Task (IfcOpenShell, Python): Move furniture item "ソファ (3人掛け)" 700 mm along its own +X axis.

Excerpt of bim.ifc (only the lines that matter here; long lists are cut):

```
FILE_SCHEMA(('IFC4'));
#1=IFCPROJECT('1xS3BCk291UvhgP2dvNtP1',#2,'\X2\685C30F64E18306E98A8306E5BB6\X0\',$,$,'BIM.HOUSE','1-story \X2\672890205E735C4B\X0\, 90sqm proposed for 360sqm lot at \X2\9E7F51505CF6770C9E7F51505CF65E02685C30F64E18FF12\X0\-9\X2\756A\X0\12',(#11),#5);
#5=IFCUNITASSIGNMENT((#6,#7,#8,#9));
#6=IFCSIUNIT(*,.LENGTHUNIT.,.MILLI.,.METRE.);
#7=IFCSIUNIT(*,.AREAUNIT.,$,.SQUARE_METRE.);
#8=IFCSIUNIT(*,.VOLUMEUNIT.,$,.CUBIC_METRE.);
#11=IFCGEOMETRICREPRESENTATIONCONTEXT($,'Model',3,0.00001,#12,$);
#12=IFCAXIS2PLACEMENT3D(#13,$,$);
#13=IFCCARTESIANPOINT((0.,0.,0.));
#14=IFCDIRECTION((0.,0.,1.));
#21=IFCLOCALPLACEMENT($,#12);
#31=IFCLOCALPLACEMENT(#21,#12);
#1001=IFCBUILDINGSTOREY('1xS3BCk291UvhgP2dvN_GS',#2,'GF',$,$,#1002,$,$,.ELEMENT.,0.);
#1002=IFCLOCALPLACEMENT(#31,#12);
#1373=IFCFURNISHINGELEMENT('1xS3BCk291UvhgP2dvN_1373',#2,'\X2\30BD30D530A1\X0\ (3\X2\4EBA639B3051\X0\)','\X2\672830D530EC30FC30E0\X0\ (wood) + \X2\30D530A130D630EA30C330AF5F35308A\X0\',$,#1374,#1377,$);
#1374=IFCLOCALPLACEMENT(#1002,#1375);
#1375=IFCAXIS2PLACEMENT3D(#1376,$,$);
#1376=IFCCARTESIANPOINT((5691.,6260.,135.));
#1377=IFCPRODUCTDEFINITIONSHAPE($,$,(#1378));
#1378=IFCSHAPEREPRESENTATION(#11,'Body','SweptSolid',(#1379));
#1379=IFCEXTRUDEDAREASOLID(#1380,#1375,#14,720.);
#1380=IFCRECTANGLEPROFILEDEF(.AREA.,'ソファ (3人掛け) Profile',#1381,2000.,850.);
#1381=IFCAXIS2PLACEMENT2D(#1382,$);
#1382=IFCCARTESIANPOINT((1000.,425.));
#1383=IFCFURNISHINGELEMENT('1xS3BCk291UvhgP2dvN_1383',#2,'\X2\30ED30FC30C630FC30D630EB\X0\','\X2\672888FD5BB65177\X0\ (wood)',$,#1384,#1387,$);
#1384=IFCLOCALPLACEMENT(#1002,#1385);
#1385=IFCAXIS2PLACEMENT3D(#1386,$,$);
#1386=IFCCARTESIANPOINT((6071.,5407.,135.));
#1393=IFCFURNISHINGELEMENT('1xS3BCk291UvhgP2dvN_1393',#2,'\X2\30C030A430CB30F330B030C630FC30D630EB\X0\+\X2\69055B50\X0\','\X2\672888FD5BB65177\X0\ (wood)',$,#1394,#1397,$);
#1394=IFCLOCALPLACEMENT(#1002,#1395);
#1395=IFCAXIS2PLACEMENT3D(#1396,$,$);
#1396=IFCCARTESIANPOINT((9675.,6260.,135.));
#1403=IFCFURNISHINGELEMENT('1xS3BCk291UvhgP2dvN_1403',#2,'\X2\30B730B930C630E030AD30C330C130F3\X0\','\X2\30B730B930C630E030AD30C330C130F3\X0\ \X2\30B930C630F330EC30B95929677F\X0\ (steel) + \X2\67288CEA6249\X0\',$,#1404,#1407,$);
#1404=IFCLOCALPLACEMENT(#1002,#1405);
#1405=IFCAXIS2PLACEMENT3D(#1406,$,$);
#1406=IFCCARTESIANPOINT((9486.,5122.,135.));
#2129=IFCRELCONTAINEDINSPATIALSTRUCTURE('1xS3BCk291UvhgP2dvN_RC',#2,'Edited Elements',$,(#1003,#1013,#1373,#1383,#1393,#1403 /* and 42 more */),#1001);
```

```python
import ifcopenshell
import ifcopenshell.api.geometry
import ifcopenshell.util.placement

model = ifcopenshell.open("bim.ifc")

item = model.by_guid("1xS3BCk291UvhgP2dvN_1373")
matrix = ifcopenshell.util.placement.get_local_placement(item.ObjectPlacement)
matrix[:3, 3] += matrix[:3, 0] * 700.0
ifcopenshell.api.geometry.edit_object_placement(model, product=item, matrix=matrix, is_si=False)

print(ifcopenshell.util.placement.get_local_placement(item.ObjectPlacement).round(3) + 0.0)

model.write("bim-out.ifc")
```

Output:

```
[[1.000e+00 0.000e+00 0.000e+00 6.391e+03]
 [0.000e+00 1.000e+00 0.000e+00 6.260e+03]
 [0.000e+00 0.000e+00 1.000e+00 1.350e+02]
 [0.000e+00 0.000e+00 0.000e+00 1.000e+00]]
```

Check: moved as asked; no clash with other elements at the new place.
